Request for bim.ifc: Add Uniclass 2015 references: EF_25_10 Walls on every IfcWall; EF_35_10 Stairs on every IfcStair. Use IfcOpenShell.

First a look at what the model holds.

```python
import ifcopenshell

model = ifcopenshell.open("bim.ifc")
print(model.schema)
print("classifications:", [c.Name for c in model.by_type("IfcClassification")])
for ifc_class in ("IfcDoor", "IfcRoof", "IfcStair", "IfcWall", "IfcWindow"):
    print(ifc_class, len(model.by_type(ifc_class)))
```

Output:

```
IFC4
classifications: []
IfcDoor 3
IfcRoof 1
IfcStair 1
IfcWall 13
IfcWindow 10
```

```python
import ifcopenshell
import ifcopenshell.api.classification

model = ifcopenshell.open("bim.ifc")

system = ifcopenshell.api.classification.add_classification(model, classification="Uniclass 2015")

codes = {
    "IfcWall": ("EF_25_10", "Walls"),
    "IfcStair": ("EF_35_10", "Stairs"),
}
for ifc_class, (code, name) in codes.items():
    products = model.by_type(ifc_class)
    ifcopenshell.api.classification.add_reference(
        model, products=products, classification=system, identification=code, name=name
    )
    print(code, len(products))

model.write("bim-out.ifc")
```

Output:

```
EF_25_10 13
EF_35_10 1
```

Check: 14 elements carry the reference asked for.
